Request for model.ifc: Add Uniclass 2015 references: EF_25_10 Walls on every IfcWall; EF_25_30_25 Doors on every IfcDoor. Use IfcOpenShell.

First a look at what the model holds.

```python
import ifcopenshell

model = ifcopenshell.open("model.ifc")
print(model.schema)
print("classifications:", [c.Name for c in model.by_type("IfcClassification")])
for ifc_class in ("IfcDoor", "IfcRoof", "IfcStair", "IfcWall", "IfcWindow"):
    print(ifc_class, len(model.by_type(ifc_class)))
```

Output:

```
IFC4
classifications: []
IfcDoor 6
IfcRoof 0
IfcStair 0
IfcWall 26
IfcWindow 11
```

```python
import ifcopenshell
import ifcopenshell.api.classification

model = ifcopenshell.open("model.ifc")

system = ifcopenshell.api.classification.add_classification(model, classification="Uniclass 2015")

codes = {
    "IfcWall": ("EF_25_10", "Walls"),
    "IfcDoor": ("EF_25_30_25", "Doors"),
}
for ifc_class, (code, name) in codes.items():
    products = model.by_type(ifc_class)
    ifcopenshell.api.classification.add_reference(
        model, products=products, classification=system, identification=code, name=name
    )
    print(code, len(products))

model.write("model_updated.ifc")
```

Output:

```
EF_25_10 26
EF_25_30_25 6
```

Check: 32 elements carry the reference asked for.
